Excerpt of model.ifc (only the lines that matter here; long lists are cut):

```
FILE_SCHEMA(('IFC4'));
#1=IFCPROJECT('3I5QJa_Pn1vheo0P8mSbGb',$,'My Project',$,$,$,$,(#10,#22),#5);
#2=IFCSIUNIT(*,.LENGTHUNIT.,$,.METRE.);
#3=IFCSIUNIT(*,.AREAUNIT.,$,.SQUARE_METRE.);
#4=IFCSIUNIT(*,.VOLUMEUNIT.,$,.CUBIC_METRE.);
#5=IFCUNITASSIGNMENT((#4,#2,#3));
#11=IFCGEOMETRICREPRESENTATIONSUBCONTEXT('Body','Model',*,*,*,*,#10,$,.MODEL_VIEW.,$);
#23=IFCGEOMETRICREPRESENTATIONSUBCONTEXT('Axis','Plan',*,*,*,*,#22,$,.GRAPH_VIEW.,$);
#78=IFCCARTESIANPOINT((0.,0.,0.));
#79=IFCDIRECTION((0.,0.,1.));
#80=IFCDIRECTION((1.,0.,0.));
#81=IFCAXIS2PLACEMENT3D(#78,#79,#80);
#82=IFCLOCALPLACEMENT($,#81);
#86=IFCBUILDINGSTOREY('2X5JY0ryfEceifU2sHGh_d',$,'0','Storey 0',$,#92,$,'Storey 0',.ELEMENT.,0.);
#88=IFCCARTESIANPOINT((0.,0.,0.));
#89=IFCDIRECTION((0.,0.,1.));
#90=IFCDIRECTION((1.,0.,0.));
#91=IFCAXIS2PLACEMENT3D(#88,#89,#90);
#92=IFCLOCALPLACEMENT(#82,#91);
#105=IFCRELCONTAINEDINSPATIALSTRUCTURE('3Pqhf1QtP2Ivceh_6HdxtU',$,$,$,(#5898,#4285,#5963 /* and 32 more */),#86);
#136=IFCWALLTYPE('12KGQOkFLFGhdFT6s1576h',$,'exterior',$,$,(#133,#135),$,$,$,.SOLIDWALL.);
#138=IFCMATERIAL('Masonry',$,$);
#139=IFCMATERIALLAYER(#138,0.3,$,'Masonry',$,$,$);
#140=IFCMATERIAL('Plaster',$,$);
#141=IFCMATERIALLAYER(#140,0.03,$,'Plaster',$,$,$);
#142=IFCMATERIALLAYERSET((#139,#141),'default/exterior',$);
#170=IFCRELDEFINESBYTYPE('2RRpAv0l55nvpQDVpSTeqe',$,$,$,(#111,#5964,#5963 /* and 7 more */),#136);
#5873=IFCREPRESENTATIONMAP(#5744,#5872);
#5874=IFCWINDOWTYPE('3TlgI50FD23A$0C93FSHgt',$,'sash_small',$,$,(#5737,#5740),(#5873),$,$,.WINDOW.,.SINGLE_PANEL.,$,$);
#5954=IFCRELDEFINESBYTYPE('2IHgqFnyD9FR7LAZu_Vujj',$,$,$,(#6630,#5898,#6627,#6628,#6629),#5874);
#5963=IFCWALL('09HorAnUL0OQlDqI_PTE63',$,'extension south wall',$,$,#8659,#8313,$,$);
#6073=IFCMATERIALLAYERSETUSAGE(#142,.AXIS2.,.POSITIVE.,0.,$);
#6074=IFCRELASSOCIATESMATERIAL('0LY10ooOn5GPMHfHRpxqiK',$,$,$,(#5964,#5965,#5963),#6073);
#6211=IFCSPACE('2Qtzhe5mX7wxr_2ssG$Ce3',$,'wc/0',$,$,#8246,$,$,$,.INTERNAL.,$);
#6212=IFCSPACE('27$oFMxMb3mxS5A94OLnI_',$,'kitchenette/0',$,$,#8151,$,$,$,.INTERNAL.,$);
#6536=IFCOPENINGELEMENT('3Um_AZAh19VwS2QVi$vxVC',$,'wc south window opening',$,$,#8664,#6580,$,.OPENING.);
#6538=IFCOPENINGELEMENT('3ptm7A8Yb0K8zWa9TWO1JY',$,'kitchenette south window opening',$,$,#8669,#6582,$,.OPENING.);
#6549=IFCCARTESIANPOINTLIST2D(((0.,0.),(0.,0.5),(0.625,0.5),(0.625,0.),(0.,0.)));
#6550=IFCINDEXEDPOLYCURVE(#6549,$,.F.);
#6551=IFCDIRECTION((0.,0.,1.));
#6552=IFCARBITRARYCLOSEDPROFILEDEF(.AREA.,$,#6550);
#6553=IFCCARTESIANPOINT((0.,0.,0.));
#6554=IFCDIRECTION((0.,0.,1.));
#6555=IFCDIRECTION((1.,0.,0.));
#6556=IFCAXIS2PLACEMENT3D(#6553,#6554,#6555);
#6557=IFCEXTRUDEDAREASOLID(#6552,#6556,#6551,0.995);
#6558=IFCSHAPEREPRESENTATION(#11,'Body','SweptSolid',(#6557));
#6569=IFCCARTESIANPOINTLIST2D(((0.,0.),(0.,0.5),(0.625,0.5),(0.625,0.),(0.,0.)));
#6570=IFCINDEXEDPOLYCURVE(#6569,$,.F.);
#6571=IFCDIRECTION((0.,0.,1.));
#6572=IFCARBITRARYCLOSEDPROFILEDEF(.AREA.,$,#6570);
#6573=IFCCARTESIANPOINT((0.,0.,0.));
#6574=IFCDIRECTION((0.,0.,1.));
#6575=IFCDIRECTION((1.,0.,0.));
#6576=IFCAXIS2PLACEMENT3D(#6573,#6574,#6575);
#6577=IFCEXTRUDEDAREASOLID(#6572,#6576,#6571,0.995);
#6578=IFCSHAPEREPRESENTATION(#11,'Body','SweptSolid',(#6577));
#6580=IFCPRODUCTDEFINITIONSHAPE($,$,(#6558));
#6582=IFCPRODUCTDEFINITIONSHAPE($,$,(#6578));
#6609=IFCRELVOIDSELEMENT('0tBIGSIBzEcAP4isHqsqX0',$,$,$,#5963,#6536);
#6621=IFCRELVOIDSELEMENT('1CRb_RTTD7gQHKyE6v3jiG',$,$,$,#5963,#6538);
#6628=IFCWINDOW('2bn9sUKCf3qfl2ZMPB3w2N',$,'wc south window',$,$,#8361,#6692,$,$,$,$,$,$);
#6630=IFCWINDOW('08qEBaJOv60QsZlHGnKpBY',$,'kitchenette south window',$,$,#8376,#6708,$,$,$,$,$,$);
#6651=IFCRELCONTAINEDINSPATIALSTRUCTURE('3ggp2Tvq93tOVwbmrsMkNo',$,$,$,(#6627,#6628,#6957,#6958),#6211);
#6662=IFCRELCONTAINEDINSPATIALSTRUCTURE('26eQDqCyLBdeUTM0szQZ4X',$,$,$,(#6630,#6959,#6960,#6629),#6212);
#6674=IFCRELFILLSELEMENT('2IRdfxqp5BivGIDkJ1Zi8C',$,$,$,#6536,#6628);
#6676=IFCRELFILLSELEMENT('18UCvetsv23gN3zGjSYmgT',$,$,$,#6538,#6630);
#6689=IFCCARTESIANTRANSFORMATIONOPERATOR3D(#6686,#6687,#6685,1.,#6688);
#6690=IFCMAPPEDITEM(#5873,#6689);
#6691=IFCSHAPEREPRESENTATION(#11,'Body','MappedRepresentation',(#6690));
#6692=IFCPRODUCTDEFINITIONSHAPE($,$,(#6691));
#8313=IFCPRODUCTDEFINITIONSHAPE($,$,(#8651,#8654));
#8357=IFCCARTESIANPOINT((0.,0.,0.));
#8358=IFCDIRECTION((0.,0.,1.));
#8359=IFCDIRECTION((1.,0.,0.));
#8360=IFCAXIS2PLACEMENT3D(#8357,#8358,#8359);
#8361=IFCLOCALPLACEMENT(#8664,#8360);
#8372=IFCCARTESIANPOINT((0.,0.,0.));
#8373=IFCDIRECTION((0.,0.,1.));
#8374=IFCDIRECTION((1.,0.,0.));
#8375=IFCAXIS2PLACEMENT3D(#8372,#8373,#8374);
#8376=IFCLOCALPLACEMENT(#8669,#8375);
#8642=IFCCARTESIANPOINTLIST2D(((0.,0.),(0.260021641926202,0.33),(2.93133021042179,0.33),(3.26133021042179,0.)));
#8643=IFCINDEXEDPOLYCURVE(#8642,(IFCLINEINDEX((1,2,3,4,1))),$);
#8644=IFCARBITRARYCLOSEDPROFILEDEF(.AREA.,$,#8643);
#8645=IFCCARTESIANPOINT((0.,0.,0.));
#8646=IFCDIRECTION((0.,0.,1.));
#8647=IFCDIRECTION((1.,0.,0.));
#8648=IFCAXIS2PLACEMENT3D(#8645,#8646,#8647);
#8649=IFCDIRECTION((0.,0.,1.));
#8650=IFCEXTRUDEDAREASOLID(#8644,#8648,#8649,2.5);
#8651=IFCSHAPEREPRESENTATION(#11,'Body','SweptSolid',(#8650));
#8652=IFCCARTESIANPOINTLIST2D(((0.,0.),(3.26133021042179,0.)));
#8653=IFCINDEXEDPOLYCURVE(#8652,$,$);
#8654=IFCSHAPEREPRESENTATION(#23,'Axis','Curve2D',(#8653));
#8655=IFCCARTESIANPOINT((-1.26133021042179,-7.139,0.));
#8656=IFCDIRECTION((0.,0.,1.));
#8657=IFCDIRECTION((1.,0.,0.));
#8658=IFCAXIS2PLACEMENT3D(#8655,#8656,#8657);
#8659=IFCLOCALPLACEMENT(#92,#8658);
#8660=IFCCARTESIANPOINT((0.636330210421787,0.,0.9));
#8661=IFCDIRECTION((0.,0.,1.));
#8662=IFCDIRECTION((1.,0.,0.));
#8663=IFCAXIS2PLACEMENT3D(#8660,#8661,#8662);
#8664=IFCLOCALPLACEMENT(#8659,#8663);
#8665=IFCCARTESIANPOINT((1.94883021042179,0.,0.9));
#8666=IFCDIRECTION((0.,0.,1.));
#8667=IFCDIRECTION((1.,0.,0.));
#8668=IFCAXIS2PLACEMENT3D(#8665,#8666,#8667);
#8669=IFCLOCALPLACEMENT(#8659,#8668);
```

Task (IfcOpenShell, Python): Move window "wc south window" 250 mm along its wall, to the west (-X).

```python
import ifcopenshell
import ifcopenshell.api.geometry
import ifcopenshell.util.placement
import ifcopenshell.util.unit

model = ifcopenshell.open("model.ifc")
unit_scale = ifcopenshell.util.unit.calculate_unit_scale(model)

window = model.by_id(6628)
opening = window.FillsVoids[0].RelatingOpeningElement
wall = opening.VoidsElements[0].RelatingBuildingElement

wall_matrix = ifcopenshell.util.placement.get_local_placement(wall.ObjectPlacement)
shift = wall_matrix[:3, 0] * -0.25 / unit_scale
before = ifcopenshell.util.placement.get_local_placement(window.ObjectPlacement)[:3, 3].copy()

# The window is placed relative to its opening, so it follows when the opening moves.
matrix = ifcopenshell.util.placement.get_local_placement(opening.ObjectPlacement)
matrix[:3, 3] += shift
ifcopenshell.api.geometry.edit_object_placement(
    model, product=opening, matrix=matrix, is_si=False, should_transform_children=True
)

after = ifcopenshell.util.placement.get_local_placement(window.ObjectPlacement)[:3, 3]
print("window moved by", (after - before).round(3) + 0.0)

model.write("model-out.ifc")
```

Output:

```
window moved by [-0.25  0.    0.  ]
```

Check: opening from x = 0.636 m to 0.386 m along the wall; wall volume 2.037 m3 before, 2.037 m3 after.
